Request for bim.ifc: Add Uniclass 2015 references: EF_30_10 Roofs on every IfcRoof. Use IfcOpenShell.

First a look at what the model holds.

```python
import ifcopenshell

model = ifcopenshell.open("bim.ifc")
print(model.schema)
print("classifications:", [c.Name for c in model.by_type("IfcClassification")])
for ifc_class in ("IfcDoor", "IfcRoof", "IfcStair", "IfcWall", "IfcWindow"):
    print(ifc_class, len(model.by_type(ifc_class)))
```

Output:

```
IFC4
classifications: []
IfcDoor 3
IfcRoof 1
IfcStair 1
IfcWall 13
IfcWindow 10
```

```python
import ifcopenshell
import ifcopenshell.api.classification

model = ifcopenshell.open("bim.ifc")

system = ifcopenshell.api.classification.add_classification(model, classification="Uniclass 2015")

codes = {
    "IfcRoof": ("EF_30_10", "Roofs"),
}
for ifc_class, (code, name) in codes.items():
    products = model.by_type(ifc_class)
    ifcopenshell.api.classification.add_reference(
        model, products=products, classification=system, identification=code, name=name
    )
    print(code, len(products))

model.write("bim_edited.ifc")
```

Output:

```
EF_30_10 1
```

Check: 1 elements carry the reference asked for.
